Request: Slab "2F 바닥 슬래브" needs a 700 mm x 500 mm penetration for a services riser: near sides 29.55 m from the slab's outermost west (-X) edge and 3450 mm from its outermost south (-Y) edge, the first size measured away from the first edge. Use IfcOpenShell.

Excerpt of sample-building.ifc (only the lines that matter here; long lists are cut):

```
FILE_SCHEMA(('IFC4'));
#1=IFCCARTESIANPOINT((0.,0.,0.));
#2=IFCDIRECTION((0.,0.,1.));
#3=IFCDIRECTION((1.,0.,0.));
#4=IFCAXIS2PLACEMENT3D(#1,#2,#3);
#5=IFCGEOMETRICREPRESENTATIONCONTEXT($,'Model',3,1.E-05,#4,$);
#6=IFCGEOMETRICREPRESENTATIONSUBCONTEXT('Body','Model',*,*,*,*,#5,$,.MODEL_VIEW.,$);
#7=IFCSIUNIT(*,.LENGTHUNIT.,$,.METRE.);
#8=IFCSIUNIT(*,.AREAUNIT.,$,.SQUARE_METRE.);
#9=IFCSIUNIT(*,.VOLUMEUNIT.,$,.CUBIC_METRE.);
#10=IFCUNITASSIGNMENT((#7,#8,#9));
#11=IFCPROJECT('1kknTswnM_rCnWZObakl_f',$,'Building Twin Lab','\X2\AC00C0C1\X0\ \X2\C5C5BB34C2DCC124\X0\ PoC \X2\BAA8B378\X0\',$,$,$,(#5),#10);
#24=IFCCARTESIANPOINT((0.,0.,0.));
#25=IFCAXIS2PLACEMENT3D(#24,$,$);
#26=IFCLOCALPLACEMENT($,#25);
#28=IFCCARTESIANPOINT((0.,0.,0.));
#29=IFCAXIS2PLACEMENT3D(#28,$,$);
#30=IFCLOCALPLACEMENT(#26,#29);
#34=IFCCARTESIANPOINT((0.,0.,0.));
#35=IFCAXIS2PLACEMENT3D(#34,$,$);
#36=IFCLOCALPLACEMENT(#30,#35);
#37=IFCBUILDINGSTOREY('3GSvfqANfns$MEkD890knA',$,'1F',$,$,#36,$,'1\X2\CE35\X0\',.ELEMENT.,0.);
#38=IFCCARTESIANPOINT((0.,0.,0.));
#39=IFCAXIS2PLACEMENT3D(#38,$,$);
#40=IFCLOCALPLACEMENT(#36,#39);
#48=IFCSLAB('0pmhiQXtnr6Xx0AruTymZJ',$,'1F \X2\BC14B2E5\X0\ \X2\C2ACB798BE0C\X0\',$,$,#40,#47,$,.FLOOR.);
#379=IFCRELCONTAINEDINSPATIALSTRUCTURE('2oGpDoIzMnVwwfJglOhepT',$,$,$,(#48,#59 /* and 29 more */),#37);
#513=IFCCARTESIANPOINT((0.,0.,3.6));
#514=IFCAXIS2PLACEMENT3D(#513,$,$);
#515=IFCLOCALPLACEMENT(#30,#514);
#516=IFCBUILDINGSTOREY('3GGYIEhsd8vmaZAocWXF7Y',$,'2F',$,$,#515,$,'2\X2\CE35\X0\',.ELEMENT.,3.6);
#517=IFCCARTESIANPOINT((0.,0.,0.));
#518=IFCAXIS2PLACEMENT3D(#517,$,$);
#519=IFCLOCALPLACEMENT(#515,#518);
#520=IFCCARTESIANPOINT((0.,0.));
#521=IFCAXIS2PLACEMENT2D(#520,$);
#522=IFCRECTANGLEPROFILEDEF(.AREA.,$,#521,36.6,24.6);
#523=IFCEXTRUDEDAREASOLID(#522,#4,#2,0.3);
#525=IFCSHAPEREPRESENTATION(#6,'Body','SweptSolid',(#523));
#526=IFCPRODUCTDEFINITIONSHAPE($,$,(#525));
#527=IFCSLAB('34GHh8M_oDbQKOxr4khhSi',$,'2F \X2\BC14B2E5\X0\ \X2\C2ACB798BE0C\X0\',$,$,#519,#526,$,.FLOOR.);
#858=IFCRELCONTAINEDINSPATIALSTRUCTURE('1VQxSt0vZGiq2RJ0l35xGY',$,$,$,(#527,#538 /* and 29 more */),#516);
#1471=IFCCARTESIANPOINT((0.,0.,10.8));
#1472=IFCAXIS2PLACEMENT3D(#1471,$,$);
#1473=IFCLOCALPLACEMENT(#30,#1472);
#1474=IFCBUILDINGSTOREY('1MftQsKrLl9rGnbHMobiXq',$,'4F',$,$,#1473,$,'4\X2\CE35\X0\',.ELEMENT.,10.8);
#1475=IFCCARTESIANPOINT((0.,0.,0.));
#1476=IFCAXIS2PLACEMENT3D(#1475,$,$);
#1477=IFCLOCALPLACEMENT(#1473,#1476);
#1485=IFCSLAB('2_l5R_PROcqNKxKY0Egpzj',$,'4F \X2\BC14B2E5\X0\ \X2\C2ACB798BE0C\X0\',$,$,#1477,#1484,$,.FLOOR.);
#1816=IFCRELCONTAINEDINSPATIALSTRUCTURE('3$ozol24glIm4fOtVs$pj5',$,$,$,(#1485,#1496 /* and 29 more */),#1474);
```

```python
import numpy as np
import ifcopenshell
import ifcopenshell.api.feature
import ifcopenshell.api.geometry
import ifcopenshell.api.root
import ifcopenshell.geom
import ifcopenshell.util.placement
import ifcopenshell.util.representation
import ifcopenshell.util.shape
import ifcopenshell.util.unit

model = ifcopenshell.open("sample-building.ifc")
unit_scale = ifcopenshell.util.unit.calculate_unit_scale(model)
settings = ifcopenshell.geom.settings()


def volume(element):
    """Net volume in cubic metres, openings subtracted."""
    shape = ifcopenshell.geom.create_shape(settings, element)
    return ifcopenshell.util.shape.get_volume(shape.geometry)


slab = model.by_guid("34GHh8M_oDbQKOxr4khhSi")
before = volume(slab)

# Extent in the slab's own axes, in metres. The edges named are its -X and -Y sides.
slab_shape = ifcopenshell.geom.create_shape(settings, slab)
vertices = ifcopenshell.util.shape.get_vertices(slab_shape.geometry)
x_min, y_min, bottom = vertices.min(axis=0)
top = vertices[:, 2].max()

opening = ifcopenshell.api.root.create_entity(model, ifc_class="IfcOpeningElement", name="Services riser opening", predefined_type="OPENING")
context = ifcopenshell.util.representation.get_context(model, "Model", "Body", "MODEL_VIEW")
width, depth = 0.7, 0.5
outline = [(0.0, 0.0), (width, 0.0), (width, depth), (0.0, depth), (0.0, 0.0)]
# Overshoot both faces by 50 mm so the cut is clean.
shape = ifcopenshell.api.geometry.add_slab_representation(
    model, context=context, depth=top - bottom + 0.1, polyline=outline
)
ifcopenshell.api.geometry.assign_representation(model, product=opening, representation=shape)

matrix = ifcopenshell.util.placement.get_local_placement(slab.ObjectPlacement)
matrix[:, 3] = matrix @ np.append(np.array([x_min + 29.55, y_min + 3.45, bottom - 0.05]) / unit_scale, 1.0)
ifcopenshell.api.geometry.edit_object_placement(model, product=opening, matrix=matrix, is_si=False)
ifcopenshell.api.feature.add_feature(model, feature=opening, element=slab)

after = volume(slab)

print(f"slab volume {before:.3f} -> {after:.3f} m3")

model.write("sample-building_v2.ifc")
```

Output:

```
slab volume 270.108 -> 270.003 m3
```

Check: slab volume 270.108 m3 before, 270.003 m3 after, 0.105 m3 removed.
